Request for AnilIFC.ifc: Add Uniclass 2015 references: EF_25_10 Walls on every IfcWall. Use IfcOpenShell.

First a look at what the model holds.

```python
import ifcopenshell

model = ifcopenshell.open("AnilIFC.ifc")
print(model.schema)
print("classifications:", [c.Name for c in model.by_type("IfcClassification")])
for ifc_class in ("IfcDoor", "IfcRoof", "IfcStair", "IfcWall", "IfcWindow"):
    print(ifc_class, len(model.by_type(ifc_class)))
```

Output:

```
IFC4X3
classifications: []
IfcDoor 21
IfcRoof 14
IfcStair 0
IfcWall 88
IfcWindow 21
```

```python
import ifcopenshell
import ifcopenshell.api.classification

model = ifcopenshell.open("AnilIFC.ifc")

system = ifcopenshell.api.classification.add_classification(model, classification="Uniclass 2015")

codes = {
    "IfcWall": ("EF_25_10", "Walls"),
}
for ifc_class, (code, name) in codes.items():
    products = model.by_type(ifc_class)
    ifcopenshell.api.classification.add_reference(
        model, products=products, classification=system, identification=code, name=name
    )
    print(code, len(products))

model.write("AnilIFC_v2.ifc")
```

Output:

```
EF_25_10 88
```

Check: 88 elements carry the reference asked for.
